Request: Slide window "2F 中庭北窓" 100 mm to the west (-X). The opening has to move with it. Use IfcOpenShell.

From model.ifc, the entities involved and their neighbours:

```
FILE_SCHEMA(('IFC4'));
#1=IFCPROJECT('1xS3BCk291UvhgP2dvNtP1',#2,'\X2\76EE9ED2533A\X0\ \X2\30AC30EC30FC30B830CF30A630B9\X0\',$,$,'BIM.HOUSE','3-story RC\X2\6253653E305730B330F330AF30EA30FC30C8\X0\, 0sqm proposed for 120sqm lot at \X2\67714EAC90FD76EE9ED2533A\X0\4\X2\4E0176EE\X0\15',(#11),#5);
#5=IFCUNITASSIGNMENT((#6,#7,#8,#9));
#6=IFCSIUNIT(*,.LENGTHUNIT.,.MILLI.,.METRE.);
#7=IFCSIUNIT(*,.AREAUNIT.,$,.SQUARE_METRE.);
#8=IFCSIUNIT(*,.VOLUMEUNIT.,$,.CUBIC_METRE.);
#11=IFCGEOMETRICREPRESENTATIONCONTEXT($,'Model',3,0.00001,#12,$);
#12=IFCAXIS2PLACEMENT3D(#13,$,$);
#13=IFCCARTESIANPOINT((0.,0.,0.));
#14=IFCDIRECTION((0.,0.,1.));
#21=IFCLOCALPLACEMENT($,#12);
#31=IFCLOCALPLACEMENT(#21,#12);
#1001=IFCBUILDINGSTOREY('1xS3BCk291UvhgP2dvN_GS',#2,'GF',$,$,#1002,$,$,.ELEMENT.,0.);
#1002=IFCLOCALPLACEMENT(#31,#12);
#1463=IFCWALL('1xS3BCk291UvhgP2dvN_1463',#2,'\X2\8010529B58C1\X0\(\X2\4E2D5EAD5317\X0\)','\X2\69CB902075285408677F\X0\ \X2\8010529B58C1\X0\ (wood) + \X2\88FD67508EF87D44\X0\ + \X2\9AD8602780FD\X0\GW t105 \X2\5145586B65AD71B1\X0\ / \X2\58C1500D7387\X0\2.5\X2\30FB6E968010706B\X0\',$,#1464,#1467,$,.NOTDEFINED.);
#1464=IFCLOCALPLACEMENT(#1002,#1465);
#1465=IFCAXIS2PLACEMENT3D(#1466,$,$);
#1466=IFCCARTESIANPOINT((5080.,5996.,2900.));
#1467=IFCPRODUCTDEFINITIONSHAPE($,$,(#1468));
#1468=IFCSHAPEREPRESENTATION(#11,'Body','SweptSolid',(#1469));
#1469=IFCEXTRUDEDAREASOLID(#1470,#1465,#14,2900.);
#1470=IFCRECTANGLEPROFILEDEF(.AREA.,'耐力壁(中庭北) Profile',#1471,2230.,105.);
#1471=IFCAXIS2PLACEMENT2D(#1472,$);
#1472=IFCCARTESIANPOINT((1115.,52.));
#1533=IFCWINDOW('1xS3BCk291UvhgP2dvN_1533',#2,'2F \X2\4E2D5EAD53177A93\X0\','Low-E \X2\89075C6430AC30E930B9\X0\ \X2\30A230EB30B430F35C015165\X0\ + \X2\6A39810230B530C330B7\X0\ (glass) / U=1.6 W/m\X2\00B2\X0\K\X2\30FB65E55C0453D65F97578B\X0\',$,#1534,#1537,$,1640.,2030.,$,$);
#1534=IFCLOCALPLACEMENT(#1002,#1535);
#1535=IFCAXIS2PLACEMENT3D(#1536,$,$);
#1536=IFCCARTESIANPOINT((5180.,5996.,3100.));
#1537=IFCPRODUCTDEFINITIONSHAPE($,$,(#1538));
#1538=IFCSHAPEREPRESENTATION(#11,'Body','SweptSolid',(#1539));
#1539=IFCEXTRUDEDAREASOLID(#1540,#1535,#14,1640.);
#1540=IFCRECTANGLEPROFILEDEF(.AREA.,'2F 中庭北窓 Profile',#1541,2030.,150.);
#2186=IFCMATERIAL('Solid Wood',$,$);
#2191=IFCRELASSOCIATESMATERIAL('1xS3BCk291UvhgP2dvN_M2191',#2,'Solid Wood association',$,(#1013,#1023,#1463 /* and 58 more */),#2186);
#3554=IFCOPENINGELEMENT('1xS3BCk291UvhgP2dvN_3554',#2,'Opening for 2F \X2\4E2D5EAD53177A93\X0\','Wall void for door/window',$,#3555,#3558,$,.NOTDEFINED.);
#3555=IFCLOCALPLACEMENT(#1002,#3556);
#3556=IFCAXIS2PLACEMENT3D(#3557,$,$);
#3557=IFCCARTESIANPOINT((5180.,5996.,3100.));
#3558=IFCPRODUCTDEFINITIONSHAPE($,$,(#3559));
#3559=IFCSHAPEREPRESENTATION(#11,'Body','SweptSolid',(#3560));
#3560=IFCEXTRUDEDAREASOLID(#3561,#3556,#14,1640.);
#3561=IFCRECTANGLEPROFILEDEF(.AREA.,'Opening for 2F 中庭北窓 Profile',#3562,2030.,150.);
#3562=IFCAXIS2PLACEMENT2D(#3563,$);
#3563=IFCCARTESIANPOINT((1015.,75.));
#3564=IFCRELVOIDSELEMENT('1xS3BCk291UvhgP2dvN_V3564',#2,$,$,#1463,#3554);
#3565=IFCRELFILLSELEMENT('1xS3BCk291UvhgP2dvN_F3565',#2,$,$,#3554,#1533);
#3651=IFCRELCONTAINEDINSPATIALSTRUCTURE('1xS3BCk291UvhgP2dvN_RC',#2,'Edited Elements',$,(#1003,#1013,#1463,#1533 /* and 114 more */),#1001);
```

```python
import ifcopenshell
import ifcopenshell.api.geometry
import ifcopenshell.util.placement
import ifcopenshell.util.unit

model = ifcopenshell.open("model.ifc")
unit_scale = ifcopenshell.util.unit.calculate_unit_scale(model)

window = model.by_guid("1xS3BCk291UvhgP2dvN_1533")
opening = window.FillsVoids[0].RelatingOpeningElement
wall = opening.VoidsElements[0].RelatingBuildingElement

wall_matrix = ifcopenshell.util.placement.get_local_placement(wall.ObjectPlacement)
shift = wall_matrix[:3, 0] * -0.1 / unit_scale
before = ifcopenshell.util.placement.get_local_placement(window.ObjectPlacement)[:3, 3].copy()

# The window is not placed relative to its opening, so move both.
for product in (opening, window):
    matrix = ifcopenshell.util.placement.get_local_placement(product.ObjectPlacement)
    matrix[:3, 3] += shift
    ifcopenshell.api.geometry.edit_object_placement(model, product=product, matrix=matrix, is_si=False)

after = ifcopenshell.util.placement.get_local_placement(window.ObjectPlacement)[:3, 3]
print("window moved by", (after - before).round(3) + 0.0)

model.write("model_updated.ifc")
```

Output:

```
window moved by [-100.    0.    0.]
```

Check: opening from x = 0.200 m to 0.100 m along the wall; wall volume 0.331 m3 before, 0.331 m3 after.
